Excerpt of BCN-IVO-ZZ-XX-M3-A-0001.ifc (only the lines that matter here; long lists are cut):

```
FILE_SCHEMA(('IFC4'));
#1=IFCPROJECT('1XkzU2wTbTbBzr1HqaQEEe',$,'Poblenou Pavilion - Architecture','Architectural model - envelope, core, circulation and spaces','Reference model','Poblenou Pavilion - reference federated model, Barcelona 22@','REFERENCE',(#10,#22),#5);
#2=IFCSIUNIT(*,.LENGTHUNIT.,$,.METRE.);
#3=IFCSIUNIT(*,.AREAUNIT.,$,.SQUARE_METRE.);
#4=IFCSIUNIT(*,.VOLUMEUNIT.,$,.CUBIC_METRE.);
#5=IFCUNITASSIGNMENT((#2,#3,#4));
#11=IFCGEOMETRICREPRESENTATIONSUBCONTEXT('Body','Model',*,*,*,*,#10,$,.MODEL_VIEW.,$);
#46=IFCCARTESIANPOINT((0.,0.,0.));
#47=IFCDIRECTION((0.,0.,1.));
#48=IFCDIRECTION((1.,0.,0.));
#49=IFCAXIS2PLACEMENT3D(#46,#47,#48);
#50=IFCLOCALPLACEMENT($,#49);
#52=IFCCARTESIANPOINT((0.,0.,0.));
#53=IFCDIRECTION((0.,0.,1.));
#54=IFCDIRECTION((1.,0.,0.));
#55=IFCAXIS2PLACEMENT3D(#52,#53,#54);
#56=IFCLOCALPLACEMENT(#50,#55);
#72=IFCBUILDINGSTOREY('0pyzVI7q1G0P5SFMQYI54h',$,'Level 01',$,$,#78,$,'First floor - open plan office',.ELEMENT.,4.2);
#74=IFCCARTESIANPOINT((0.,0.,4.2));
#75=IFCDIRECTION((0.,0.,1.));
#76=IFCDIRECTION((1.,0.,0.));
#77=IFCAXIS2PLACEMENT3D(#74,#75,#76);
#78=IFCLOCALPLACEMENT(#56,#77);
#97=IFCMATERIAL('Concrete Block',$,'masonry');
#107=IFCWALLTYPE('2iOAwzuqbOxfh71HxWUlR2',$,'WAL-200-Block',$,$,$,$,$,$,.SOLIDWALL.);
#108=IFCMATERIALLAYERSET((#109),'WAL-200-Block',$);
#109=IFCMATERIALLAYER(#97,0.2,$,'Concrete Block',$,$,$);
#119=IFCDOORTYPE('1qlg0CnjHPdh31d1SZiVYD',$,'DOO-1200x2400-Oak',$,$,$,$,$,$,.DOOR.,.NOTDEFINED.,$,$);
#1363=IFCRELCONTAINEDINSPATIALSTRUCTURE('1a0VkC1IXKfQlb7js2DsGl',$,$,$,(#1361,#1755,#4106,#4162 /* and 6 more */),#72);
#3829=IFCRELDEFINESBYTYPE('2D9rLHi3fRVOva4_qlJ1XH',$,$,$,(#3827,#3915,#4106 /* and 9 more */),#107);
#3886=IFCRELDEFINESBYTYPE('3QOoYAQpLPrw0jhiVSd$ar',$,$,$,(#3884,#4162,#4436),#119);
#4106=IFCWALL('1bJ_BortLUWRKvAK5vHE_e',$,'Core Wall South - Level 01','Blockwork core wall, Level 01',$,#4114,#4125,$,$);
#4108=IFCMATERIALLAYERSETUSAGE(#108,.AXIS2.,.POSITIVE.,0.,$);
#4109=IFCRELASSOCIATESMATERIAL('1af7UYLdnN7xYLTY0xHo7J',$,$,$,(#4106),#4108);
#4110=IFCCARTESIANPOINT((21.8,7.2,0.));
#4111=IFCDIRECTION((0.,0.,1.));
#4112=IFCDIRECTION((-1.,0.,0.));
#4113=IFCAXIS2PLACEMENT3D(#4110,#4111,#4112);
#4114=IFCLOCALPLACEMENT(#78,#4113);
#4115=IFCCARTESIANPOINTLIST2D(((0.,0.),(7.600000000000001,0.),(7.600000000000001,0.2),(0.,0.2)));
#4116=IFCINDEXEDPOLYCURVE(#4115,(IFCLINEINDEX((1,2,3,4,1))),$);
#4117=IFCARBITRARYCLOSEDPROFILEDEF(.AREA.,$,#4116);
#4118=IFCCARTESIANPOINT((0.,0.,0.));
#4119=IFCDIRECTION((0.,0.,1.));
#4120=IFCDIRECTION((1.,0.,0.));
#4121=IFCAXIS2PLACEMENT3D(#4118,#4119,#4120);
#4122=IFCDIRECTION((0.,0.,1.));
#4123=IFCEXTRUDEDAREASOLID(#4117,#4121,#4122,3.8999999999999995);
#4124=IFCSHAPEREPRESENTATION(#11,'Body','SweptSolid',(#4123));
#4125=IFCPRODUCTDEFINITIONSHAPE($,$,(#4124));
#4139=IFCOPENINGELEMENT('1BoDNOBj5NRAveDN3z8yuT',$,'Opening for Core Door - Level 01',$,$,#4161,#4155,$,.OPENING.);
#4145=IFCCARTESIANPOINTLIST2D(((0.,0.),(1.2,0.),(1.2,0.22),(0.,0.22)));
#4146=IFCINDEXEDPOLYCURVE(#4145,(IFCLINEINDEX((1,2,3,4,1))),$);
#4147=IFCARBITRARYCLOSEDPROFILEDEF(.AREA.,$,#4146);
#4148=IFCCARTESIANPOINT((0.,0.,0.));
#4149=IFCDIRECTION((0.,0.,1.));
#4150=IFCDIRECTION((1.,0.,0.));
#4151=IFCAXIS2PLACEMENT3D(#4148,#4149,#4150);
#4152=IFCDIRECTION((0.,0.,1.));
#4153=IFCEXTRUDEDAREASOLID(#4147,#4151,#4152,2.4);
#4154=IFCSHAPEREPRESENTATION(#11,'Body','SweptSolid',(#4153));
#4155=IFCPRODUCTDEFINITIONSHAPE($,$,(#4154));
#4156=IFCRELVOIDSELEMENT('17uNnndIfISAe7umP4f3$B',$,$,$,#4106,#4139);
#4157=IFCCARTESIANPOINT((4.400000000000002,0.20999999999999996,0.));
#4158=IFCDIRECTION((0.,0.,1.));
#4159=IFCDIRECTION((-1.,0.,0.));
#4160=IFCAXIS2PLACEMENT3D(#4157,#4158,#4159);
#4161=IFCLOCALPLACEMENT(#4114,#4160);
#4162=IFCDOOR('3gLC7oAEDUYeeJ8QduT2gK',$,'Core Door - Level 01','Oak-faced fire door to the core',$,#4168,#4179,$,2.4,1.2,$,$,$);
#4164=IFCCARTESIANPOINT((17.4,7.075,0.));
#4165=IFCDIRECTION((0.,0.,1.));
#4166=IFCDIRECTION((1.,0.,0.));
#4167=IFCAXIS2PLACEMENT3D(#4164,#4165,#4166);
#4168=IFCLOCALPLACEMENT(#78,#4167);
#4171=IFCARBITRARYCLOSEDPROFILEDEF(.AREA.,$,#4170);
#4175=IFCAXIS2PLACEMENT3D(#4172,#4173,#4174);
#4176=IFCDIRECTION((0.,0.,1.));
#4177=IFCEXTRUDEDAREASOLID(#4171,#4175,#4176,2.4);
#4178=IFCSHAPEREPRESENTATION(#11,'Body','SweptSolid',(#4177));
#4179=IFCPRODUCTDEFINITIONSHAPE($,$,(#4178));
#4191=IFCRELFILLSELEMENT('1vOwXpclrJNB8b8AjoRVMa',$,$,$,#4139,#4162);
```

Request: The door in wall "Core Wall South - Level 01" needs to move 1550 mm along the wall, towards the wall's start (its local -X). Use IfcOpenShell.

```python
import ifcopenshell
import ifcopenshell.api.geometry
import ifcopenshell.util.placement
import ifcopenshell.util.unit

model = ifcopenshell.open("BCN-IVO-ZZ-XX-M3-A-0001.ifc")
unit_scale = ifcopenshell.util.unit.calculate_unit_scale(model)

door = model.by_id(4162)
opening = door.FillsVoids[0].RelatingOpeningElement
wall = opening.VoidsElements[0].RelatingBuildingElement

wall_matrix = ifcopenshell.util.placement.get_local_placement(wall.ObjectPlacement)
shift = wall_matrix[:3, 0] * -1.55 / unit_scale
before = ifcopenshell.util.placement.get_local_placement(door.ObjectPlacement)[:3, 3].copy()

# The door is not placed relative to its opening, so move both.
for product in (opening, door):
    matrix = ifcopenshell.util.placement.get_local_placement(product.ObjectPlacement)
    matrix[:3, 3] += shift
    ifcopenshell.api.geometry.edit_object_placement(model, product=product, matrix=matrix, is_si=False)

after = ifcopenshell.util.placement.get_local_placement(door.ObjectPlacement)[:3, 3]
print("door moved by", (after - before).round(3) + 0.0)

model.write("BCN-IVO-ZZ-XX-M3-A-0001_v2.ifc")
```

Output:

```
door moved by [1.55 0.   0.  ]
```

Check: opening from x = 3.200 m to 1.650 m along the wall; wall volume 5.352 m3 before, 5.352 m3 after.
